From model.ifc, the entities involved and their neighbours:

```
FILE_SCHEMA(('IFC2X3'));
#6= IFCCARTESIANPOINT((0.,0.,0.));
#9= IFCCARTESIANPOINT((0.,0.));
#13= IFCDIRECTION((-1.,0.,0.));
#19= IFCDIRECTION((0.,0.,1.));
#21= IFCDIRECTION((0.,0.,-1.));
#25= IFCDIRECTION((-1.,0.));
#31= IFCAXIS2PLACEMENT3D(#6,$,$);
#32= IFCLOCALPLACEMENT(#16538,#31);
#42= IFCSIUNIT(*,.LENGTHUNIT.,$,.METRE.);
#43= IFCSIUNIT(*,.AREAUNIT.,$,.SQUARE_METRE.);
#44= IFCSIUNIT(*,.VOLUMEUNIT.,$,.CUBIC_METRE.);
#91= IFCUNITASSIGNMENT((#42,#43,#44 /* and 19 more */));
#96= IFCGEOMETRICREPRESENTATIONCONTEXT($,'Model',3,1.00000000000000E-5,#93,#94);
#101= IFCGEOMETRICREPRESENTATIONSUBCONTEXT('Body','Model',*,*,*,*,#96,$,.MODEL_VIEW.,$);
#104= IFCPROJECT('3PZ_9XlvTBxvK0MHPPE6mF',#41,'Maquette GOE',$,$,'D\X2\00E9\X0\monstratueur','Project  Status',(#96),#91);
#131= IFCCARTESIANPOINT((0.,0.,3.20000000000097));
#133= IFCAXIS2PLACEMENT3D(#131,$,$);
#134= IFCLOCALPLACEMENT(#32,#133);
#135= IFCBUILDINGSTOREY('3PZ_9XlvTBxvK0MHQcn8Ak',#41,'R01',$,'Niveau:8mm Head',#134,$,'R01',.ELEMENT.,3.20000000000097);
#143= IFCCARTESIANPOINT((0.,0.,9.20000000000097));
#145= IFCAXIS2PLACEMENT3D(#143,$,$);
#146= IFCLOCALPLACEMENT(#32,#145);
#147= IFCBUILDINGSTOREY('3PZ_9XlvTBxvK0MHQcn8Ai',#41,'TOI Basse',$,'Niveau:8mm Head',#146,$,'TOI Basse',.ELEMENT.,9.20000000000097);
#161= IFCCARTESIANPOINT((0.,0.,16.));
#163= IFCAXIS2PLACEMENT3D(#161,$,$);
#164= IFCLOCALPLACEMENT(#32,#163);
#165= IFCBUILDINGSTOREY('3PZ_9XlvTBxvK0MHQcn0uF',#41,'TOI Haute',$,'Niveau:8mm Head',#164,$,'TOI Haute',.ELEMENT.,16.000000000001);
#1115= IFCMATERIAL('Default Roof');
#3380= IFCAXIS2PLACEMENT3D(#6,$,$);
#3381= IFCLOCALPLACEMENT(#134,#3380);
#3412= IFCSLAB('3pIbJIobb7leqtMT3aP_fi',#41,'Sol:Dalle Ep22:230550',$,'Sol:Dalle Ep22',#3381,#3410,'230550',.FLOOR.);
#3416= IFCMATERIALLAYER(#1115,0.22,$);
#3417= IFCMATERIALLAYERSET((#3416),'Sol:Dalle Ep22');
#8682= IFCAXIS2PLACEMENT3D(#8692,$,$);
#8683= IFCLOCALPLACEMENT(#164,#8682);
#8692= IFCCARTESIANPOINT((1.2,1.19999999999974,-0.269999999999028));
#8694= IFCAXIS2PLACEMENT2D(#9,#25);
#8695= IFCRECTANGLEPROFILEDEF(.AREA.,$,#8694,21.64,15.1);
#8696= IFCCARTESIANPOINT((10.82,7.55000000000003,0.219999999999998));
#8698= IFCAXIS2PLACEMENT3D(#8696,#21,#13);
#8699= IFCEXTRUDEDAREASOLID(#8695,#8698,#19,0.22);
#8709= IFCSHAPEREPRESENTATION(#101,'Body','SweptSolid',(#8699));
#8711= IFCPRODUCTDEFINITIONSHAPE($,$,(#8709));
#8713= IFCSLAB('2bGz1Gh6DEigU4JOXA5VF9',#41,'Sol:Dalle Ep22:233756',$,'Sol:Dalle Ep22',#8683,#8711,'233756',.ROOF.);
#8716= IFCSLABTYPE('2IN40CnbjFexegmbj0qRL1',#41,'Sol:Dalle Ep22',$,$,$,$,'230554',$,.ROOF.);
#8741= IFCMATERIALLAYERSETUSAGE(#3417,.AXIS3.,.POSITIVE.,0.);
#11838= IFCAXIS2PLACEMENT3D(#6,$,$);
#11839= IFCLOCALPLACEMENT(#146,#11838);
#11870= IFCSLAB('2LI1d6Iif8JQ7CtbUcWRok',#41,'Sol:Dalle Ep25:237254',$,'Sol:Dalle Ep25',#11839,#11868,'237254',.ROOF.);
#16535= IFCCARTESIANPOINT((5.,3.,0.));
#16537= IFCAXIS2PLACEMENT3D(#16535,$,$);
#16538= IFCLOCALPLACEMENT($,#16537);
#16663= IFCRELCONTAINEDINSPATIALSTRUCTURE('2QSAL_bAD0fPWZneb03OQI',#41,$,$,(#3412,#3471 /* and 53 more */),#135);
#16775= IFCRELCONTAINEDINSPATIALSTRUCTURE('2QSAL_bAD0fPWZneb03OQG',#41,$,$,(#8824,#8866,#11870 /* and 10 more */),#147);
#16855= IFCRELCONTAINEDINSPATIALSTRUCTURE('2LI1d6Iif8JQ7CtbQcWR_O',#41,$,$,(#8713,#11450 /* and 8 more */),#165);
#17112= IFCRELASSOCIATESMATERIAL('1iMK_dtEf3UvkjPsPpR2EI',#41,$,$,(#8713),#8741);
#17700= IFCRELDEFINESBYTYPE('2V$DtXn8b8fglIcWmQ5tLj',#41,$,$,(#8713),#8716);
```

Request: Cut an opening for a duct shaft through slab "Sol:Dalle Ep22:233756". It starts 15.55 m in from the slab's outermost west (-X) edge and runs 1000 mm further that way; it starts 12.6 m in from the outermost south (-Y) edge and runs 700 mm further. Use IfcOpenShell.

```python
import numpy as np
import ifcopenshell
import ifcopenshell.api.feature
import ifcopenshell.api.geometry
import ifcopenshell.api.root
import ifcopenshell.geom
import ifcopenshell.util.placement
import ifcopenshell.util.representation
import ifcopenshell.util.shape
import ifcopenshell.util.unit

model = ifcopenshell.open("model.ifc")
unit_scale = ifcopenshell.util.unit.calculate_unit_scale(model)
settings = ifcopenshell.geom.settings()


def volume(element):
    """Net volume in cubic metres, openings subtracted."""
    shape = ifcopenshell.geom.create_shape(settings, element)
    return ifcopenshell.util.shape.get_volume(shape.geometry)


slab = model.by_guid("2bGz1Gh6DEigU4JOXA5VF9")
before = volume(slab)

# Extent in the slab's own axes, in metres. The edges named are its -X and -Y sides.
slab_shape = ifcopenshell.geom.create_shape(settings, slab)
vertices = ifcopenshell.util.shape.get_vertices(slab_shape.geometry)
x_min, y_min, bottom = vertices.min(axis=0)
top = vertices[:, 2].max()

opening = ifcopenshell.api.root.create_entity(model, ifc_class="IfcOpeningElement", name="Duct shaft opening")
context = ifcopenshell.util.representation.get_context(model, "Model", "Body", "MODEL_VIEW")
width, depth = 1, 0.7
outline = [(0.0, 0.0), (width, 0.0), (width, depth), (0.0, depth), (0.0, 0.0)]
# Overshoot both faces by 50 mm so the cut is clean.
shape = ifcopenshell.api.geometry.add_slab_representation(
    model, context=context, depth=top - bottom + 0.1, polyline=outline
)
ifcopenshell.api.geometry.assign_representation(model, product=opening, representation=shape)

matrix = ifcopenshell.util.placement.get_local_placement(slab.ObjectPlacement)
matrix[:, 3] = matrix @ np.append(np.array([x_min + 15.55, y_min + 12.6, bottom - 0.05]) / unit_scale, 1.0)
ifcopenshell.api.geometry.edit_object_placement(model, product=opening, matrix=matrix, is_si=False)
ifcopenshell.api.feature.add_feature(model, feature=opening, element=slab)

after = volume(slab)

print(f"slab volume {before:.3f} -> {after:.3f} m3")

model.write("model_v2.ifc")
```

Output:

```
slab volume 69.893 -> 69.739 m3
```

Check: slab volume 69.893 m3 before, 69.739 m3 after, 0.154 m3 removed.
